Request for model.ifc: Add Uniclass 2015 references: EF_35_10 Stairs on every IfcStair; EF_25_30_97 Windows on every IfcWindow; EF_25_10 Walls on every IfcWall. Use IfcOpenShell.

First a look at what the model holds.

```python
import ifcopenshell

model = ifcopenshell.open("model.ifc")
print(model.schema)
print("classifications:", [c.Name for c in model.by_type("IfcClassification")])
for ifc_class in ("IfcDoor", "IfcRoof", "IfcStair", "IfcWall", "IfcWindow"):
    print(ifc_class, len(model.by_type(ifc_class)))
```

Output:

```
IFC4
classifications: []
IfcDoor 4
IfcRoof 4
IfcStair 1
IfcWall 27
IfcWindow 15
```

```python
import ifcopenshell
import ifcopenshell.api.classification

model = ifcopenshell.open("model.ifc")

system = ifcopenshell.api.classification.add_classification(model, classification="Uniclass 2015")

codes = {
    "IfcStair": ("EF_35_10", "Stairs"),
    "IfcWindow": ("EF_25_30_97", "Windows"),
    "IfcWall": ("EF_25_10", "Walls"),
}
for ifc_class, (code, name) in codes.items():
    products = model.by_type(ifc_class)
    ifcopenshell.api.classification.add_reference(
        model, products=products, classification=system, identification=code, name=name
    )
    print(code, len(products))

model.write("model_v2.ifc")
```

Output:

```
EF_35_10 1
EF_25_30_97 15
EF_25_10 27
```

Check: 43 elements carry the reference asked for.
